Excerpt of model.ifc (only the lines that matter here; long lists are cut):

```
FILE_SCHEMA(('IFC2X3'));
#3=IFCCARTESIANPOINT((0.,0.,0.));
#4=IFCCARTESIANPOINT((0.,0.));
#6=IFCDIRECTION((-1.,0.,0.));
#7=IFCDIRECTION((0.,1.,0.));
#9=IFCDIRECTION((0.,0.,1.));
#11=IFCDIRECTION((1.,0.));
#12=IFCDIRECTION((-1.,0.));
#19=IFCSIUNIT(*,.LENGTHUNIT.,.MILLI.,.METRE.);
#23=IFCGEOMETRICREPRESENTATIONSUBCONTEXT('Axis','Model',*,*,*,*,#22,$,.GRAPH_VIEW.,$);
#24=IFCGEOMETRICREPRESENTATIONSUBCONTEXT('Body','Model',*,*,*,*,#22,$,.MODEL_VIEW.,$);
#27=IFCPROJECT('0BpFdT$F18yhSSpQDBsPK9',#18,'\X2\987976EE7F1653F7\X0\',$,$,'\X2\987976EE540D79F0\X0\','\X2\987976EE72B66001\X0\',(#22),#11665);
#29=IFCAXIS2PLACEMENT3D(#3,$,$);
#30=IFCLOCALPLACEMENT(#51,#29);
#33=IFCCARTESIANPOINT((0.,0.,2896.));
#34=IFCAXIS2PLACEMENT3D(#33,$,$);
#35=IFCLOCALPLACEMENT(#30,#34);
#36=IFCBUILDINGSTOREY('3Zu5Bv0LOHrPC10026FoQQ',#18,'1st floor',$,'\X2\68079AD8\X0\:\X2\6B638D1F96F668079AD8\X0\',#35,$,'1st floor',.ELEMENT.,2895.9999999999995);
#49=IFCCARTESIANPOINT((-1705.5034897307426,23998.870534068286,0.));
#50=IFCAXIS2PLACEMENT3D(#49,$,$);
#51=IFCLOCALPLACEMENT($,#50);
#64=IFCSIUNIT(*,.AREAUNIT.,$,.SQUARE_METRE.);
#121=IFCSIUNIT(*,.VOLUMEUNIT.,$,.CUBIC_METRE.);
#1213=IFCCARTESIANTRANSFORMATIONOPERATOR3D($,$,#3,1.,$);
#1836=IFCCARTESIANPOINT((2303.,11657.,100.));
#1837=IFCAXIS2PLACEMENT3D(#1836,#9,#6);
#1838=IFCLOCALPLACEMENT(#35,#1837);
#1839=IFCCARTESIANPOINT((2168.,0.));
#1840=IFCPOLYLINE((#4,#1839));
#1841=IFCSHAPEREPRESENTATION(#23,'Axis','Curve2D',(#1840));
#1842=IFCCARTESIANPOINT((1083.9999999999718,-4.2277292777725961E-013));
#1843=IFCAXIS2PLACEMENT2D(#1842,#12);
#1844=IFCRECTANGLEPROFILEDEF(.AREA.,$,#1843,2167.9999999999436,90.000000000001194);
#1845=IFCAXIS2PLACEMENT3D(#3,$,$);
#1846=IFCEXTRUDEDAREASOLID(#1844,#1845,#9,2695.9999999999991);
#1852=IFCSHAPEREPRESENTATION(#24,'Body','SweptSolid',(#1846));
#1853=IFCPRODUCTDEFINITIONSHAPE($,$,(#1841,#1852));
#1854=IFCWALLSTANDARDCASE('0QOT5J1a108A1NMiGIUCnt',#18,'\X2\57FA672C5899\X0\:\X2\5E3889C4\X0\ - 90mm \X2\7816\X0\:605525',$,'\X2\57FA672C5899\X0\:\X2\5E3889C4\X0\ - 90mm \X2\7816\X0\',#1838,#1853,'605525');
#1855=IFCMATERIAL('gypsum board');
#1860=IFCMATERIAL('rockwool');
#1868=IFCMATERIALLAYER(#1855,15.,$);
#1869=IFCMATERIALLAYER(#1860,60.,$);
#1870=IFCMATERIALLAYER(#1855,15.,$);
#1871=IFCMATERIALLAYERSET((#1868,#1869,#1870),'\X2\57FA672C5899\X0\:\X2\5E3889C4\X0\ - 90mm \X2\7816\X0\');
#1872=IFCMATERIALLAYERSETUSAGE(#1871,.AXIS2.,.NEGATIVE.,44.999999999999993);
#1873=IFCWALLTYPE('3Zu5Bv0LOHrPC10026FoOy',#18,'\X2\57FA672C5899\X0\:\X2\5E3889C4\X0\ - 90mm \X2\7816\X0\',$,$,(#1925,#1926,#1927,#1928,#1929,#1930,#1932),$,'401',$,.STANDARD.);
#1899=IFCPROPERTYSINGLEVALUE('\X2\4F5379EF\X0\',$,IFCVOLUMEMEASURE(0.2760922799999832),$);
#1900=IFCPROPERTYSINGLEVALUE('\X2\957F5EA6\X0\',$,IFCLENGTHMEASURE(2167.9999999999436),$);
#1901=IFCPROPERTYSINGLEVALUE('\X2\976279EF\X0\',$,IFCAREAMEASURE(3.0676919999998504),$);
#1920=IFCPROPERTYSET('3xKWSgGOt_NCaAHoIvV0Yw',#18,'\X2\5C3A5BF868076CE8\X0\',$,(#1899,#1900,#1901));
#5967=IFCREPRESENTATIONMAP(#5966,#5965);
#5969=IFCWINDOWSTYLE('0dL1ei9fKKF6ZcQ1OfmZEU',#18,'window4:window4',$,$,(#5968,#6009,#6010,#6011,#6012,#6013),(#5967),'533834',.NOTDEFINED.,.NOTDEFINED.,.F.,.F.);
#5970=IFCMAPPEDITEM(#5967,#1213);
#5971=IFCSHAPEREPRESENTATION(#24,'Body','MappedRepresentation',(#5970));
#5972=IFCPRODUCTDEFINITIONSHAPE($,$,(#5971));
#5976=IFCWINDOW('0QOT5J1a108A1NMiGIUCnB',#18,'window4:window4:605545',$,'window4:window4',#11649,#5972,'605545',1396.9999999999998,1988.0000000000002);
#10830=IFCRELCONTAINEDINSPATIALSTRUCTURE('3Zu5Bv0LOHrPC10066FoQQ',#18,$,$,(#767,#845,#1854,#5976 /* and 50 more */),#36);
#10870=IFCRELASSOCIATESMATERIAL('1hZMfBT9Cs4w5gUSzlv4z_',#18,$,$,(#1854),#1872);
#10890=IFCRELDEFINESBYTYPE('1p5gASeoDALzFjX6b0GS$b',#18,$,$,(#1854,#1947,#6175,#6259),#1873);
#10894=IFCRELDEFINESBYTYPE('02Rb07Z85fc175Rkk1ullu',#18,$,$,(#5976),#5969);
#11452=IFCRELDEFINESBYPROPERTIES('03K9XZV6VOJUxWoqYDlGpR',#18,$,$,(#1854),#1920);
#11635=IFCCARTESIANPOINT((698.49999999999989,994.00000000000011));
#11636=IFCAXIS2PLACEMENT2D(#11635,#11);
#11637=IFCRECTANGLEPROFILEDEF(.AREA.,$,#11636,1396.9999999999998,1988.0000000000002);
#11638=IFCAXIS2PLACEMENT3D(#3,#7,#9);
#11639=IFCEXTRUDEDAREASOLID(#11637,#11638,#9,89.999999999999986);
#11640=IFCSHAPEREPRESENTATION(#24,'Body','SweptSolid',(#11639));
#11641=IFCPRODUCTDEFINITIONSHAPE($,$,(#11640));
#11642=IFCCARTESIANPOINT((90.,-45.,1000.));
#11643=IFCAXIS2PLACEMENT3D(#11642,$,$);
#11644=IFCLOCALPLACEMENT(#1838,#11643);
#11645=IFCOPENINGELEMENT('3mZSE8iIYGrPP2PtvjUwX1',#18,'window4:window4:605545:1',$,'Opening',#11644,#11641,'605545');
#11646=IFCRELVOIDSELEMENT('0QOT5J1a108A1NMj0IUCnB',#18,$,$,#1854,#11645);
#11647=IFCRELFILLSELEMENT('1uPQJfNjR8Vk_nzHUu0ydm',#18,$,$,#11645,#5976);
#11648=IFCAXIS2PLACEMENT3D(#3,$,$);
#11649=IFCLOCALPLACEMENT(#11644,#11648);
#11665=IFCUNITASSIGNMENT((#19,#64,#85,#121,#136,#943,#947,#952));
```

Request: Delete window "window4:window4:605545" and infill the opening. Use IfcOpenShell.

```python
import ifcopenshell
import ifcopenshell.api.feature
import ifcopenshell.api.pset
import ifcopenshell.api.root
import ifcopenshell.geom
import ifcopenshell.util.element
import ifcopenshell.util.shape
import ifcopenshell.util.unit

model = ifcopenshell.open("model.ifc")
area_scale = ifcopenshell.util.unit.calculate_unit_scale(model, "AREAUNIT")
volume_scale = ifcopenshell.util.unit.calculate_unit_scale(model, "VOLUMEUNIT")
settings = ifcopenshell.geom.settings()


def volume(element):
    """Net volume in cubic metres, openings subtracted."""
    shape = ifcopenshell.geom.create_shape(settings, element)
    return ifcopenshell.util.shape.get_volume(shape.geometry)


window = model.by_guid("0QOT5J1a108A1NMiGIUCnB")
opening = window.FillsVoids[0].RelatingOpeningElement
wall = opening.VoidsElements[0].RelatingBuildingElement
before = volume(wall)

ifcopenshell.api.root.remove_product(model, product=window)
ifcopenshell.api.feature.remove_feature(model, feature=opening)

after = volume(wall)
thickness = 0.09  # wall thickness in metres

# Update the wall's stored quantities.
pset = model.by_id(ifcopenshell.util.element.get_pset(wall, "尺寸标注", should_inherit=False)["id"])
ifcopenshell.api.pset.edit_pset(model, pset=pset, properties={
    "体积": model.create_entity("IfcVolumeMeasure", after / volume_scale),
    "面积": model.create_entity("IfcAreaMeasure", after / thickness / area_scale),
})

print(f"wall volume {before:.3f} -> {after:.3f} m3")

model.write("model-out.ifc")
```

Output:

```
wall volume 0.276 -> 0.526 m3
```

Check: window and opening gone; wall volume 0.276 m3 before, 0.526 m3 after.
